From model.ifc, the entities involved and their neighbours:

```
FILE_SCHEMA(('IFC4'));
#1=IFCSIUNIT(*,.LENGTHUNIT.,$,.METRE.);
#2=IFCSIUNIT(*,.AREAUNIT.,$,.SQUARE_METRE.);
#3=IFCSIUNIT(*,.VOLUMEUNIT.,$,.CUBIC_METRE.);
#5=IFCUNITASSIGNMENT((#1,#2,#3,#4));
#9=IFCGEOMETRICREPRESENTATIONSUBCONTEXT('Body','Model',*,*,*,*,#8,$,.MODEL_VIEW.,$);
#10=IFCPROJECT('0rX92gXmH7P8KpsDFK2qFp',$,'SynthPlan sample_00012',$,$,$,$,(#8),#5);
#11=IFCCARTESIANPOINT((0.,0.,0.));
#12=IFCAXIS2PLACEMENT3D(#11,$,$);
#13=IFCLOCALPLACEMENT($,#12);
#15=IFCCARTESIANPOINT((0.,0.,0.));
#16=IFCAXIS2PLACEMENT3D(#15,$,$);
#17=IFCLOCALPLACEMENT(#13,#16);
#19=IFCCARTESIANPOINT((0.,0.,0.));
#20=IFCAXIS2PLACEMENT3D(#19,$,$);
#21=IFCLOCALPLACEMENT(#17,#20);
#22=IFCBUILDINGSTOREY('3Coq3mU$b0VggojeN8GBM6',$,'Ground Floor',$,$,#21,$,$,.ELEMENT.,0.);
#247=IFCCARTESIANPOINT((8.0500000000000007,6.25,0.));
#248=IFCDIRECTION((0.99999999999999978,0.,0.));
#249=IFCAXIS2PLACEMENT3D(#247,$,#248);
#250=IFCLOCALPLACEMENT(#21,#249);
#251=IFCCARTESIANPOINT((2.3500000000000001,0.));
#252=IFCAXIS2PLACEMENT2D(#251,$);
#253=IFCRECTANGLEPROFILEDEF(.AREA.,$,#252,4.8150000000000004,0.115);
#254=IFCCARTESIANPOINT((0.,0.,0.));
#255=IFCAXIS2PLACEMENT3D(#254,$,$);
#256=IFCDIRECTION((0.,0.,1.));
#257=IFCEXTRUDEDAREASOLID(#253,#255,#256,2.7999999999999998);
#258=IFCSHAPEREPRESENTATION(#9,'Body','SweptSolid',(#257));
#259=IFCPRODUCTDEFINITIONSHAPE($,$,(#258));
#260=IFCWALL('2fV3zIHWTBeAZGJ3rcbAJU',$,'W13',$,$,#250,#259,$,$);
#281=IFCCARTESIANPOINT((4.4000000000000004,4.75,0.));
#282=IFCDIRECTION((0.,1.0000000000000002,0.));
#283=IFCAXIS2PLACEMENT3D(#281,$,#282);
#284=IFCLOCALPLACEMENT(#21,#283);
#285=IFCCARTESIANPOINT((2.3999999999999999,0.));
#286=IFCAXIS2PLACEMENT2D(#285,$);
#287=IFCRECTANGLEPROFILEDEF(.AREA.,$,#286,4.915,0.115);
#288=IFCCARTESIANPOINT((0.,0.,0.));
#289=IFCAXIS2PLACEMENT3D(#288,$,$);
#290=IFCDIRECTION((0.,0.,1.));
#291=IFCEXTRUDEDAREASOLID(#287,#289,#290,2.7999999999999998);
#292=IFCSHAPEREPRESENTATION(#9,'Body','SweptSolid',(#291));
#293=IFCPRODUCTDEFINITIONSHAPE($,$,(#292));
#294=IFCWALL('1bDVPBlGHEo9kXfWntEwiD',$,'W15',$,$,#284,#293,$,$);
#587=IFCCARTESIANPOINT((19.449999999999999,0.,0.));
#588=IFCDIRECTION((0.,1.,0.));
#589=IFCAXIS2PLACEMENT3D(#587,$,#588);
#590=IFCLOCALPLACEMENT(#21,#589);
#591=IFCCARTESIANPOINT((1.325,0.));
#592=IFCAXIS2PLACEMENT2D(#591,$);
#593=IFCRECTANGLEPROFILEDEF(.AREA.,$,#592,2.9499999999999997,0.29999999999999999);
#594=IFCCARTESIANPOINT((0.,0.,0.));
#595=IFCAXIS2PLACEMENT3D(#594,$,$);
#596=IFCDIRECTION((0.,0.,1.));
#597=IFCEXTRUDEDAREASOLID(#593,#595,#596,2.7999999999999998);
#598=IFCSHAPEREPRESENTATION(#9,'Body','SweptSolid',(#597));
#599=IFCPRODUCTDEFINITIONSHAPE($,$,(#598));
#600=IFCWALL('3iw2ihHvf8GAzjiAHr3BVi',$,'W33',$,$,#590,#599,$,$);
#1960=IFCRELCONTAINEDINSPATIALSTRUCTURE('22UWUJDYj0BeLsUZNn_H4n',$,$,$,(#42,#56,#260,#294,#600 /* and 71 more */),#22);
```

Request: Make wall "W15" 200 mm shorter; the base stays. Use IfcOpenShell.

```python
import ifcopenshell
import ifcopenshell.geom
import ifcopenshell.util.representation
import ifcopenshell.util.shape
import ifcopenshell.util.unit

model = ifcopenshell.open("model.ifc")
unit_scale = ifcopenshell.util.unit.calculate_unit_scale(model)
settings = ifcopenshell.geom.settings()


def volume(element):
    """Net volume in cubic metres, openings subtracted."""
    shape = ifcopenshell.geom.create_shape(settings, element)
    return ifcopenshell.util.shape.get_volume(shape.geometry)


wall = model.by_guid("1bDVPBlGHEo9kXfWntEwiD")
before = volume(wall)

body = ifcopenshell.util.representation.get_representation(wall, "Model", "Body")
solid = body.Items[0]
old_height = solid.Depth
solid.Depth -= 0.2 / unit_scale
after = volume(wall)

print(f"height {old_height:g} -> {solid.Depth:g}, volume {before:.3f} -> {after:.3f} m3")

model.write("model-out.ifc")
```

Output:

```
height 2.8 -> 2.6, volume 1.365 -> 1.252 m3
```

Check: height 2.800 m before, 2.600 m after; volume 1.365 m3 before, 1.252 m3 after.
